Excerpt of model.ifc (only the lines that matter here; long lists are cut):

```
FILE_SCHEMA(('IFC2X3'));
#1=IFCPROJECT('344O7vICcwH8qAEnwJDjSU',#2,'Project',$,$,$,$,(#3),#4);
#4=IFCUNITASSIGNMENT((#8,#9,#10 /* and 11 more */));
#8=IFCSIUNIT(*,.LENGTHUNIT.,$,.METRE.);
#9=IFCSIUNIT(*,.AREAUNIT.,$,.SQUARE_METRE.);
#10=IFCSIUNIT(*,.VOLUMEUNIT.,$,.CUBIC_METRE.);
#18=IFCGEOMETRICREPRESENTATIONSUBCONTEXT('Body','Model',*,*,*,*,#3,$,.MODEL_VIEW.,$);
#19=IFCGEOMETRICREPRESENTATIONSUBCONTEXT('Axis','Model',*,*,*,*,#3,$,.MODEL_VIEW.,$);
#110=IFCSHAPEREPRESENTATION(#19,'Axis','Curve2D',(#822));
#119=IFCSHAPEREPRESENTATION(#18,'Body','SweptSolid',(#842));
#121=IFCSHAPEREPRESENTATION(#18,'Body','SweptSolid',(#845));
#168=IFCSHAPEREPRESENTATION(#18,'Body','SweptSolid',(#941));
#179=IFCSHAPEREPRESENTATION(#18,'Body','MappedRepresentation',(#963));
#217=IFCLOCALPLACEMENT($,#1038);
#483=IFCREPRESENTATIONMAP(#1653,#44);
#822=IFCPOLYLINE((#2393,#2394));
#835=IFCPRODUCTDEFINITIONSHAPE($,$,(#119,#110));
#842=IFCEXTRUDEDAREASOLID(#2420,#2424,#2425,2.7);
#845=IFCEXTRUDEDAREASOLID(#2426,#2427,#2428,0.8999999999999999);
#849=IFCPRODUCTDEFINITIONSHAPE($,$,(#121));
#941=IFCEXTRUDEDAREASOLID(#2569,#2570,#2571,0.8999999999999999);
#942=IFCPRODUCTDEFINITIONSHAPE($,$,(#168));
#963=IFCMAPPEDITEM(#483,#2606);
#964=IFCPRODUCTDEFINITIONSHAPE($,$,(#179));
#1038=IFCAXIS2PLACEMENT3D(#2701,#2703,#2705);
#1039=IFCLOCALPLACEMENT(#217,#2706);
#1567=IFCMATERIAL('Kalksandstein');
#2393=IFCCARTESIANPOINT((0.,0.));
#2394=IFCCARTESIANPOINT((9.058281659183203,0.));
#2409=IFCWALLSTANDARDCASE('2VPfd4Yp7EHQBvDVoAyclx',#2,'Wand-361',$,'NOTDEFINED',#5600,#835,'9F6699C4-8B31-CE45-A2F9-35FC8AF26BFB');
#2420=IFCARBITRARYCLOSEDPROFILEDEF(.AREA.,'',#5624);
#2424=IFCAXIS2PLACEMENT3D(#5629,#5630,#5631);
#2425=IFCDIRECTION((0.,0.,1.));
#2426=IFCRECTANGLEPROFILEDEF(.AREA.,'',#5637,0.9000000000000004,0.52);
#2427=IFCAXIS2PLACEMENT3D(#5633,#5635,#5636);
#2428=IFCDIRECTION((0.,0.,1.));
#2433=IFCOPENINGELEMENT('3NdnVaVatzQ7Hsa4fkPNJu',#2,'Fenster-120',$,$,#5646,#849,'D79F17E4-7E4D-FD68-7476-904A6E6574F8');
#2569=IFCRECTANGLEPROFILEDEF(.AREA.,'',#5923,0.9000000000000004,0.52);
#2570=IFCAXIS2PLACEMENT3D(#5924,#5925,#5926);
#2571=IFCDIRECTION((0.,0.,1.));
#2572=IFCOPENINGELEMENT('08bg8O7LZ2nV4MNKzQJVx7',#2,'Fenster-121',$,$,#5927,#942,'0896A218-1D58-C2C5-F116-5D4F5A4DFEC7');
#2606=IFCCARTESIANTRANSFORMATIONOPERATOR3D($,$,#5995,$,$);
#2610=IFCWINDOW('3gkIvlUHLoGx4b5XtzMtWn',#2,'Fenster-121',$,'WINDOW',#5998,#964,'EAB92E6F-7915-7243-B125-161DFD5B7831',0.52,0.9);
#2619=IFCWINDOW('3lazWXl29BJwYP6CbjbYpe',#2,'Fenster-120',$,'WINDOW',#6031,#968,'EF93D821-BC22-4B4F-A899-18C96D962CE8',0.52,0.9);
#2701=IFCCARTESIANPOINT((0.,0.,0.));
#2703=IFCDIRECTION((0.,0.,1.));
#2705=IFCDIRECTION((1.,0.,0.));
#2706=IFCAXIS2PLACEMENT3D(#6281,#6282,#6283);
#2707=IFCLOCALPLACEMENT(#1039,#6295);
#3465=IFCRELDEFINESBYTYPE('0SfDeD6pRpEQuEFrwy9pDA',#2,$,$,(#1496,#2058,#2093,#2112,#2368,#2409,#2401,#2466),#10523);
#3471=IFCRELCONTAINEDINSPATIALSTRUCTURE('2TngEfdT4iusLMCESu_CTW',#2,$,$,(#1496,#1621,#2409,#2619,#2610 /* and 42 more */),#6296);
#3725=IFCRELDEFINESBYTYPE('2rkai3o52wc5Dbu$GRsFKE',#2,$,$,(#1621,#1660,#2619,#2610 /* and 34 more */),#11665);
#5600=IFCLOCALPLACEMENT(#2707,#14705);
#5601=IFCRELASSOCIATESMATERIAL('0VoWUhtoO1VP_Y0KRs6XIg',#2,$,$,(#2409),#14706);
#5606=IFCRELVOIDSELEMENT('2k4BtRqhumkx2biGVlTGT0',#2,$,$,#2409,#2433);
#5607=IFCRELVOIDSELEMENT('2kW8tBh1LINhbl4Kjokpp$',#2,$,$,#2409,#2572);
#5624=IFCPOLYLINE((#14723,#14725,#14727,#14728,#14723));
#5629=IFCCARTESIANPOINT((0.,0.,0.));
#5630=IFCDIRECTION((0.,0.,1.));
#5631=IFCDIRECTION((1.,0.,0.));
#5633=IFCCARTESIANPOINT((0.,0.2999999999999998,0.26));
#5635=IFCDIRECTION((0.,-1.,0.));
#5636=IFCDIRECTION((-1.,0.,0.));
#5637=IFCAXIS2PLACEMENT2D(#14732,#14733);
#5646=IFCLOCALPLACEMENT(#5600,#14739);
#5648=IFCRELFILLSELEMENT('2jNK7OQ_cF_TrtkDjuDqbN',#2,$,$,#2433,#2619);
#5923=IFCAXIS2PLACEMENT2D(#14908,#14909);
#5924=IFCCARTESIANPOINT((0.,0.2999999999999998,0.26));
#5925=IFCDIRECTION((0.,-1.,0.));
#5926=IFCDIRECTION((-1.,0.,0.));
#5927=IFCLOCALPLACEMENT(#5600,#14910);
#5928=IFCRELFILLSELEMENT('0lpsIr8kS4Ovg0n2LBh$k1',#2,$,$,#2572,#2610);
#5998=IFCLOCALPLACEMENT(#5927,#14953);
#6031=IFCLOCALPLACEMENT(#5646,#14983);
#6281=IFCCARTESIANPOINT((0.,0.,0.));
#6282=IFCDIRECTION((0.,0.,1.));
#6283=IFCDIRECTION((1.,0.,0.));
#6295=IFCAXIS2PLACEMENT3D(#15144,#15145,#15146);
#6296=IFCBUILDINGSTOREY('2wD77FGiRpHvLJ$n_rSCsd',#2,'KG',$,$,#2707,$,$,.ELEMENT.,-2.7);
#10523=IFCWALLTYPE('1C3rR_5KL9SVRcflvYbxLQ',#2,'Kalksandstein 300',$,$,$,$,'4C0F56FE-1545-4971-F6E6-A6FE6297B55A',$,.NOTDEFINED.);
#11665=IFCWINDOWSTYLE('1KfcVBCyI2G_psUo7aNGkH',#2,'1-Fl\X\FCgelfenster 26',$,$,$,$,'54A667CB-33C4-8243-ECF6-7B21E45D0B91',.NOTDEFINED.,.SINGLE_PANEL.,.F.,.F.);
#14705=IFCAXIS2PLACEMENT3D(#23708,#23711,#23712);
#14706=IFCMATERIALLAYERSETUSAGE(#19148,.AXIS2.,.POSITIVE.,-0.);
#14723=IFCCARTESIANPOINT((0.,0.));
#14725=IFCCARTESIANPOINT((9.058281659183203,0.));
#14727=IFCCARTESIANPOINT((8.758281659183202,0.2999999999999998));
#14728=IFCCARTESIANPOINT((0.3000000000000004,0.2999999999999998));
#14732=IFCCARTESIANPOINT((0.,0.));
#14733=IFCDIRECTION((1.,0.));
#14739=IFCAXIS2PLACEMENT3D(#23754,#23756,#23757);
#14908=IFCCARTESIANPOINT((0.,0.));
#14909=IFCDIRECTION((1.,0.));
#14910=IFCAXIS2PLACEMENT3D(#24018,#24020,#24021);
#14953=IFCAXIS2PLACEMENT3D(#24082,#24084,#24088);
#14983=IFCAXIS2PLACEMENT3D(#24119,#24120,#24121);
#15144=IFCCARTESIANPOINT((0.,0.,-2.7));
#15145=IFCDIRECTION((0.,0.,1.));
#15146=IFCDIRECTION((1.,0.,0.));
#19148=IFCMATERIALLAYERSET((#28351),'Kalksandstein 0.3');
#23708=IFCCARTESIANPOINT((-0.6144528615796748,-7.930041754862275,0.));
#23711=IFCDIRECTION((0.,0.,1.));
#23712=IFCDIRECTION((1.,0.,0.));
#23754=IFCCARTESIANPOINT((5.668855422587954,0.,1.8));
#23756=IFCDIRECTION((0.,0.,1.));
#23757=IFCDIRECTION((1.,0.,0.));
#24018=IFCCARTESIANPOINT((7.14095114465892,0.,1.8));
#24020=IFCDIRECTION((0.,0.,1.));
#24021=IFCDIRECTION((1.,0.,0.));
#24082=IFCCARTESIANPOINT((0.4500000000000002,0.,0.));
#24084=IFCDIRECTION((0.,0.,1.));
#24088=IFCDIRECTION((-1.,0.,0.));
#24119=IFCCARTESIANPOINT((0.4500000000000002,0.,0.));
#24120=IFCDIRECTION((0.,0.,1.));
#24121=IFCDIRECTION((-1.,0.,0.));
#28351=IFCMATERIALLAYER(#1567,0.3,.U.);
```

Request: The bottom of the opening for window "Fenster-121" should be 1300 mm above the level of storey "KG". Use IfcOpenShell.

```python
import numpy as np
import ifcopenshell
import ifcopenshell.api.geometry
import ifcopenshell.geom
import ifcopenshell.util.element
import ifcopenshell.util.placement
import ifcopenshell.util.shape
import ifcopenshell.util.unit

model = ifcopenshell.open("model.ifc")
unit_scale = ifcopenshell.util.unit.calculate_unit_scale(model)

window = model.by_guid("3gkIvlUHLoGx4b5XtzMtWn")
opening = window.FillsVoids[0].RelatingOpeningElement
storey = ifcopenshell.util.element.get_container(window, ifc_class="IfcBuildingStorey")
level = ifcopenshell.util.placement.get_local_placement(storey.ObjectPlacement)[2, 3]

# The opening's origin need not be at the sill, so measure its lowest point.
shape = ifcopenshell.geom.create_shape(ifcopenshell.geom.settings(), opening)
bottom = ifcopenshell.util.shape.get_shape_bottom_elevation(shape, shape.geometry) / unit_scale
dz = level + 1.3 - bottom

shift = np.array([0.0, 0.0, dz])
# The window is placed relative to its opening, so it follows when the opening moves.
matrix = ifcopenshell.util.placement.get_local_placement(opening.ObjectPlacement)
matrix[:3, 3] += shift
ifcopenshell.api.geometry.edit_object_placement(
    model, product=opening, matrix=matrix, is_si=False, should_transform_children=True
)

print(f"moved by {dz * unit_scale:+.3f} m")

model.write("model_rev.ifc")
```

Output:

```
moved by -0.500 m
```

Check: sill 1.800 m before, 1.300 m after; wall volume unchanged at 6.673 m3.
